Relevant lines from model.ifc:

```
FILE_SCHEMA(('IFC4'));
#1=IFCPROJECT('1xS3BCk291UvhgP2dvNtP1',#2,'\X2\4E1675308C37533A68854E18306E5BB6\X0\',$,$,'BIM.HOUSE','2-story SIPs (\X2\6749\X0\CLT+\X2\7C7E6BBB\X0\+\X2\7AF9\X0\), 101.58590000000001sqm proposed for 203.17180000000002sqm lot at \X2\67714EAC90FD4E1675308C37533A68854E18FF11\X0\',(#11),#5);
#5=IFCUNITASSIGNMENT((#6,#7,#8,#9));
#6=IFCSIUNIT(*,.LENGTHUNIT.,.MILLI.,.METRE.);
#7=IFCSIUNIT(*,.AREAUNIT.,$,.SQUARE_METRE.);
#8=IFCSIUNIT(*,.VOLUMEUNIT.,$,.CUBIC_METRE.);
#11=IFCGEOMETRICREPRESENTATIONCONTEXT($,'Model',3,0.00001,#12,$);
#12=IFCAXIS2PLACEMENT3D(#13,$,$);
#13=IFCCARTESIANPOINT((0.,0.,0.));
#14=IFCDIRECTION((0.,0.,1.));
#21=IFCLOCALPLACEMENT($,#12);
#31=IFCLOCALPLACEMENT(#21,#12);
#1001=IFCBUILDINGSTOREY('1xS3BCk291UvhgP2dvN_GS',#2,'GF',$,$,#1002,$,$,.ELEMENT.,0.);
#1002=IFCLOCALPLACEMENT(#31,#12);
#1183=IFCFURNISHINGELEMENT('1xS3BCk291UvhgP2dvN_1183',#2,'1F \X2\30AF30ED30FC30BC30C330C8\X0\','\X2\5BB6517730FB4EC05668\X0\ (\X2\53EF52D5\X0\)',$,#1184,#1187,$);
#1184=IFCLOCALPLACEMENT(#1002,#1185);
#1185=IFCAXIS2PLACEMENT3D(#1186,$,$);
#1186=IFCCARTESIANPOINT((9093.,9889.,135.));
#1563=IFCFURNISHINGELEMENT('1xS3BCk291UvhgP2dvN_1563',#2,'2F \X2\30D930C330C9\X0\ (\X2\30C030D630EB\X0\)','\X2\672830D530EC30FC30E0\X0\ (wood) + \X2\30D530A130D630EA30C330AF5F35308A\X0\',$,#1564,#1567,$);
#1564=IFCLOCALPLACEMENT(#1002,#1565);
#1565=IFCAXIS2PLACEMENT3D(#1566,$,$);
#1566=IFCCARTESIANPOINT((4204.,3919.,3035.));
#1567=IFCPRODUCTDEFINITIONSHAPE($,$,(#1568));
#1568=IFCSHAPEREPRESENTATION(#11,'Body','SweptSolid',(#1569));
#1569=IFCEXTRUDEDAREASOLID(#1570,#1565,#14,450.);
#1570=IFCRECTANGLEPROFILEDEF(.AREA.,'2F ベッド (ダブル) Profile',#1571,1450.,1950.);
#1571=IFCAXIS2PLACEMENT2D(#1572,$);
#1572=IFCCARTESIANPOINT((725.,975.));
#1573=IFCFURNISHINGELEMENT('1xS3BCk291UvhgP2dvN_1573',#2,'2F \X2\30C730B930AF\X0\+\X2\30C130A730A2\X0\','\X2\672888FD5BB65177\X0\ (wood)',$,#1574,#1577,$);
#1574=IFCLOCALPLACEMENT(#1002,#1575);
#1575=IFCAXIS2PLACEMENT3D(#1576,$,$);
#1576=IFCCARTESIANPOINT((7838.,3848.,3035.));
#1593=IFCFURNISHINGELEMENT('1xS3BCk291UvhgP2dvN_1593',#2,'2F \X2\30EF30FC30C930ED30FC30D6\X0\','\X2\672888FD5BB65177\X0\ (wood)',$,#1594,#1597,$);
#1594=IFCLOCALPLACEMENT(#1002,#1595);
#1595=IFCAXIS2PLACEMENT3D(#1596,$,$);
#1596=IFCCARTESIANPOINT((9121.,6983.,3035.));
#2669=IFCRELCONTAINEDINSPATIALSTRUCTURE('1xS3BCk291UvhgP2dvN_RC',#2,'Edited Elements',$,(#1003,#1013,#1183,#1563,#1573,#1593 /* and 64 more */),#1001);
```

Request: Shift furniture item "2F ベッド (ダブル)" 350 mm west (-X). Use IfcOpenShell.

```python
import ifcopenshell
import ifcopenshell.api.geometry
import ifcopenshell.util.placement

model = ifcopenshell.open("model.ifc")

item = model.by_guid("1xS3BCk291UvhgP2dvN_1563")
matrix = ifcopenshell.util.placement.get_local_placement(item.ObjectPlacement)
matrix[0, 3] -= 350.0
ifcopenshell.api.geometry.edit_object_placement(model, product=item, matrix=matrix, is_si=False)

print(ifcopenshell.util.placement.get_local_placement(item.ObjectPlacement).round(3) + 0.0)

model.write("model-out.ifc")
```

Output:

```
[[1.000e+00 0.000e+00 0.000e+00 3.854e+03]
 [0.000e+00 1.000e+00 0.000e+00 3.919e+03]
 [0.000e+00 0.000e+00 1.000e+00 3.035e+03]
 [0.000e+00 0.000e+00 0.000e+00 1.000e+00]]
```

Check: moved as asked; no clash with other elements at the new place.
